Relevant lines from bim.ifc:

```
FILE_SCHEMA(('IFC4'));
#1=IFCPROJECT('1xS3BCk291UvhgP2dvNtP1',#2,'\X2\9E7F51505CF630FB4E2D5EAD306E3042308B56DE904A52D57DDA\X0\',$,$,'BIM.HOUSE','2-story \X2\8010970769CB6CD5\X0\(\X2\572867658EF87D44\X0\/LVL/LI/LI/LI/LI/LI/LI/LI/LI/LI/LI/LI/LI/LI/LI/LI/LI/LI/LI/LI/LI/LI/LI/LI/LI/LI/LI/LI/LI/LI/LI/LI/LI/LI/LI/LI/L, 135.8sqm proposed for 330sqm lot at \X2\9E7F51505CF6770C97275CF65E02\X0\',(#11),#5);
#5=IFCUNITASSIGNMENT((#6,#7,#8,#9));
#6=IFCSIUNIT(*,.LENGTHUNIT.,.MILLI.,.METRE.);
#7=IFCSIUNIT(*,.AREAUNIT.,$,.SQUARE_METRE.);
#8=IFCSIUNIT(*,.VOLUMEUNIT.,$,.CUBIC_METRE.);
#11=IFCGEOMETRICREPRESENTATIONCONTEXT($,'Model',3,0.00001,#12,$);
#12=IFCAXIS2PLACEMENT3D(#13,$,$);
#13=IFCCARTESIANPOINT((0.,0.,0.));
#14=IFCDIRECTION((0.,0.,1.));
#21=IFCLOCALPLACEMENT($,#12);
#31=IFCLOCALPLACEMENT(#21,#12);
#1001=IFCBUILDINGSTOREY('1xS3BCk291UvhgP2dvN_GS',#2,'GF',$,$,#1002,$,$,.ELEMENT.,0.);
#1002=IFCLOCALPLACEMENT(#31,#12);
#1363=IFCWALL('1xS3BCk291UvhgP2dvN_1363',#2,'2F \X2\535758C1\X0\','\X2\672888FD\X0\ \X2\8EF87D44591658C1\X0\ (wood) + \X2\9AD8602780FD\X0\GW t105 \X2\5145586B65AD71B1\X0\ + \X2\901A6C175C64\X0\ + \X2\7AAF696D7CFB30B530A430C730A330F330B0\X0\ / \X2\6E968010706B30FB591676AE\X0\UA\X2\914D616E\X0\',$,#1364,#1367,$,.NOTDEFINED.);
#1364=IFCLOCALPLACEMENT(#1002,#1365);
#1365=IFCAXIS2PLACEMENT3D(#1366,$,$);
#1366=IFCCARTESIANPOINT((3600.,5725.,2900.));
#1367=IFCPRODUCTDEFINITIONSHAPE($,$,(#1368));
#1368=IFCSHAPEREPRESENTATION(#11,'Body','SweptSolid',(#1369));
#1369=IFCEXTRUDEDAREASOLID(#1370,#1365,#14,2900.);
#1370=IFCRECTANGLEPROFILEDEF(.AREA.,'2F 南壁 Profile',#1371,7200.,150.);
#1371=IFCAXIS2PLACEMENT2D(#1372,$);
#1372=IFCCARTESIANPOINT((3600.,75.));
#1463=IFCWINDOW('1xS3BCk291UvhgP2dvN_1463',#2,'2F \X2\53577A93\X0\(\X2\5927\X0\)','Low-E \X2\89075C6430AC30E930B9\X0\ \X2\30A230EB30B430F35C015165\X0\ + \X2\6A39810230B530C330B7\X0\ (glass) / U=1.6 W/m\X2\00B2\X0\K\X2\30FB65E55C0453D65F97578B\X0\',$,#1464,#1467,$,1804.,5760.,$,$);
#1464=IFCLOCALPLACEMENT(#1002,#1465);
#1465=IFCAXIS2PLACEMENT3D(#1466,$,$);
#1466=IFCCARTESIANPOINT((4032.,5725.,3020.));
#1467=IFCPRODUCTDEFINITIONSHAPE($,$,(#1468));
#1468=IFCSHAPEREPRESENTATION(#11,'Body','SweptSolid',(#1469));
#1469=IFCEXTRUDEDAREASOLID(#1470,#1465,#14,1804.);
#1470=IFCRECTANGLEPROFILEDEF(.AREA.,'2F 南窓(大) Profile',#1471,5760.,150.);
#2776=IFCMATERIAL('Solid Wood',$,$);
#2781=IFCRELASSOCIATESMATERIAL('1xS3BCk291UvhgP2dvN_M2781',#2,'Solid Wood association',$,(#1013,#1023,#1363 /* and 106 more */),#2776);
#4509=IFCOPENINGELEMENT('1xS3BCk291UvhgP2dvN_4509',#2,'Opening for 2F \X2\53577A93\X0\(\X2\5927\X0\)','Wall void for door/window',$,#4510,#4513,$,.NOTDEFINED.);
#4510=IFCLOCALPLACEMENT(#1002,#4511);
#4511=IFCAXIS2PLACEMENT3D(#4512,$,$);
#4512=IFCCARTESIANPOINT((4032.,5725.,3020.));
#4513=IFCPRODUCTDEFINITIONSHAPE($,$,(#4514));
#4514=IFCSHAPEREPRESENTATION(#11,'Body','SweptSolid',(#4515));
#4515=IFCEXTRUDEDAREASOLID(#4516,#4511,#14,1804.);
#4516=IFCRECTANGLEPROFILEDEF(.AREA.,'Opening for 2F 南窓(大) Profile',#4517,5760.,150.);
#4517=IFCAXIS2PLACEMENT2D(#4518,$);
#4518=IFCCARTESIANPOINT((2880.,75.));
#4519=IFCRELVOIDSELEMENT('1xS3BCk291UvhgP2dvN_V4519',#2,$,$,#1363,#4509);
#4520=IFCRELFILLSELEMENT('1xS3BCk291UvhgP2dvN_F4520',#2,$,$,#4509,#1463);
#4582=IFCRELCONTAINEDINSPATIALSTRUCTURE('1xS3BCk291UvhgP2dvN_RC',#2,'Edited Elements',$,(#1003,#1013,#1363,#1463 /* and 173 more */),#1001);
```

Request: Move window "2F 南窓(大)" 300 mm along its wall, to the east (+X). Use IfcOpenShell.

```python
import ifcopenshell
import ifcopenshell.api.geometry
import ifcopenshell.util.placement
import ifcopenshell.util.unit

model = ifcopenshell.open("bim.ifc")
unit_scale = ifcopenshell.util.unit.calculate_unit_scale(model)

window = model.by_guid("1xS3BCk291UvhgP2dvN_1463")
opening = window.FillsVoids[0].RelatingOpeningElement
wall = opening.VoidsElements[0].RelatingBuildingElement

wall_matrix = ifcopenshell.util.placement.get_local_placement(wall.ObjectPlacement)
shift = wall_matrix[:3, 0] * 0.3 / unit_scale
before = ifcopenshell.util.placement.get_local_placement(window.ObjectPlacement)[:3, 3].copy()

# The window is not placed relative to its opening, so move both.
for product in (opening, window):
    matrix = ifcopenshell.util.placement.get_local_placement(product.ObjectPlacement)
    matrix[:3, 3] += shift
    ifcopenshell.api.geometry.edit_object_placement(model, product=product, matrix=matrix, is_si=False)

after = ifcopenshell.util.placement.get_local_placement(window.ObjectPlacement)[:3, 3]
print("window moved by", (after - before).round(3) + 0.0)

model.write("bim_updated.ifc")
```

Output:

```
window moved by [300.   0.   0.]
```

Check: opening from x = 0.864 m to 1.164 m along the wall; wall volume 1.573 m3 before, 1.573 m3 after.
